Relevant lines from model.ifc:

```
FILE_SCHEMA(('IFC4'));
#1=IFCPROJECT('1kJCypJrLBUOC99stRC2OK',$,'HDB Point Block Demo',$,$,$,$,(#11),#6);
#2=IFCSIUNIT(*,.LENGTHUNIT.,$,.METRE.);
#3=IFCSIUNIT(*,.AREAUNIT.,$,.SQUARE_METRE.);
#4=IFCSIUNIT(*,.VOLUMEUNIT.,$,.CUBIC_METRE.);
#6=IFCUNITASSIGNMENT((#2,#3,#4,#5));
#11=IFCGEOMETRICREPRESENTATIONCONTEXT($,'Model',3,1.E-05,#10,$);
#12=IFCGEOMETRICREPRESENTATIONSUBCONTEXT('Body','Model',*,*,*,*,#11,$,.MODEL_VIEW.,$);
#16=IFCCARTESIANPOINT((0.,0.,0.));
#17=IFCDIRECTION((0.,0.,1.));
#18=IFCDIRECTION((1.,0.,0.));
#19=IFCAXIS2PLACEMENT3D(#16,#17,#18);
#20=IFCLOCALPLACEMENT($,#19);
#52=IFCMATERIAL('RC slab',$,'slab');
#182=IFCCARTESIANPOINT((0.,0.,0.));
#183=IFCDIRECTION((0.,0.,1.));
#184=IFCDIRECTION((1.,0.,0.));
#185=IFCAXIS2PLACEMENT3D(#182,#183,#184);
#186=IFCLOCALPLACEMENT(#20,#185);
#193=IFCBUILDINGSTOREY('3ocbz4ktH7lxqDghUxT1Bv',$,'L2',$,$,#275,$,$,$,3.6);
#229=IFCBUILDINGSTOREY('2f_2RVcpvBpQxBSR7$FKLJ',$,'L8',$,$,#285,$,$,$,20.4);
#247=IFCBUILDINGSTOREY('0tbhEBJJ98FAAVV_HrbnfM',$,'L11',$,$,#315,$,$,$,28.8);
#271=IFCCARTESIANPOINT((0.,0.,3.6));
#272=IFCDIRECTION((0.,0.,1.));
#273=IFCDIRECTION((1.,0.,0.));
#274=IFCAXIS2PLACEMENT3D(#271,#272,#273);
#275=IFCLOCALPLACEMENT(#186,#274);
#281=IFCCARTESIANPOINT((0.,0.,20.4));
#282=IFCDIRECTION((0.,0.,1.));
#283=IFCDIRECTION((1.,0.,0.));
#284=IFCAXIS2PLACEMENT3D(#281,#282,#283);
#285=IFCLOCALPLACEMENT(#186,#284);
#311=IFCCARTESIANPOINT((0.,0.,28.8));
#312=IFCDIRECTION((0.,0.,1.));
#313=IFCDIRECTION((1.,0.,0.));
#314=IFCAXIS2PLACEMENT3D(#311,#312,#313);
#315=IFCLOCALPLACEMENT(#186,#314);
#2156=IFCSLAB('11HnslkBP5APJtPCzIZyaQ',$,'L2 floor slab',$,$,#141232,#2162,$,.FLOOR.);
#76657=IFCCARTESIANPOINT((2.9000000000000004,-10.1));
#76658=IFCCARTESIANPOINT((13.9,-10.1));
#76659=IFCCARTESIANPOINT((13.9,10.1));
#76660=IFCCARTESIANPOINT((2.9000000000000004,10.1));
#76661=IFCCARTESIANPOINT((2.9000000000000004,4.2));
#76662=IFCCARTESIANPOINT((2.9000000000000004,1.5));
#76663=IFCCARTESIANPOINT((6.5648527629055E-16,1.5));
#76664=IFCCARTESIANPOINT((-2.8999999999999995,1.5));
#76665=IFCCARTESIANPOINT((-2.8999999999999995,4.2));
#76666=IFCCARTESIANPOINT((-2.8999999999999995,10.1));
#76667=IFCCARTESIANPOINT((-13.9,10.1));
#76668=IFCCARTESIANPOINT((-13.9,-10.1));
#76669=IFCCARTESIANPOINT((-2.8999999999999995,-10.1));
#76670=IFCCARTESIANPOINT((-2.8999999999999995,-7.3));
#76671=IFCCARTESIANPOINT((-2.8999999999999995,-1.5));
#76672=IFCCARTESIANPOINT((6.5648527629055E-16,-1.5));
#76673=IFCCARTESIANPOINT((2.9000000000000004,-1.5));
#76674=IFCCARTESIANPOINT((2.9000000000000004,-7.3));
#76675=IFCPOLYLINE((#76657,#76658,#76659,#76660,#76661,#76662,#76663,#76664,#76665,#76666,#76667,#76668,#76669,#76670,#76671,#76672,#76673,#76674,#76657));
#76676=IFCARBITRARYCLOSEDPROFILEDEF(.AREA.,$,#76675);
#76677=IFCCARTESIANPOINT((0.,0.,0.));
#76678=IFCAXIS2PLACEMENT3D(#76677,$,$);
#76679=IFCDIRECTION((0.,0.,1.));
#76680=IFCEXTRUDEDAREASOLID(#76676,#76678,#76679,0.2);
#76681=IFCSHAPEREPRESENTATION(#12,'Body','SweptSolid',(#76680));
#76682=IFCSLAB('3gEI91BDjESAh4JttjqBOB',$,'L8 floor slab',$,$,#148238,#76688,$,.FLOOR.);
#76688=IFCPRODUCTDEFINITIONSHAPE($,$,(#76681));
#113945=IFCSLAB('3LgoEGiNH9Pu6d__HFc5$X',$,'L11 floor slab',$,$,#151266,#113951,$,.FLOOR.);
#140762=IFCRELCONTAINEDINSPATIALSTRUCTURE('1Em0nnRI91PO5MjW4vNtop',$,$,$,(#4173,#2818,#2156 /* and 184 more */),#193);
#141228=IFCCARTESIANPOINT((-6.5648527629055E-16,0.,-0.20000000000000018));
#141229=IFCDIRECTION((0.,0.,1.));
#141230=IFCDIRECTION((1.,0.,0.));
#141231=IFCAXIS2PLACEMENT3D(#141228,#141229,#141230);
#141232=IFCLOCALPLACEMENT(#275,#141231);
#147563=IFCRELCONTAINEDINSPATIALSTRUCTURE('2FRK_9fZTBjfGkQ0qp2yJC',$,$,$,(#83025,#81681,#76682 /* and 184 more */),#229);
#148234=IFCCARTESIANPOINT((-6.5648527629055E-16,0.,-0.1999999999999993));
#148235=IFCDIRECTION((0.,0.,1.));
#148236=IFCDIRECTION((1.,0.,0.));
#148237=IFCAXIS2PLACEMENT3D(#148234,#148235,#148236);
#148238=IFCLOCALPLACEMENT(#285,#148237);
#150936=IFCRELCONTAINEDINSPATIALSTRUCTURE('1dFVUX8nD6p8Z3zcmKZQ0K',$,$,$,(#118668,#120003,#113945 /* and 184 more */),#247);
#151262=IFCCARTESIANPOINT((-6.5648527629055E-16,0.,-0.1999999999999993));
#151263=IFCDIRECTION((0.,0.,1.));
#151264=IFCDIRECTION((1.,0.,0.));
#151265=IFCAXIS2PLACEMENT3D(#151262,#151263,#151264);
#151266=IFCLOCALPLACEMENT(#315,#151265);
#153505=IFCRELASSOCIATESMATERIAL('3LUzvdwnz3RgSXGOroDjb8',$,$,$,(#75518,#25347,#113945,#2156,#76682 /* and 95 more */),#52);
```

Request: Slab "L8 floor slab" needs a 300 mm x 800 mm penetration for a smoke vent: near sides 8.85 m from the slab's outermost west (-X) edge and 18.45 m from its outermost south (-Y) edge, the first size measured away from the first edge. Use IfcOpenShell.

```python
import numpy as np
import ifcopenshell
import ifcopenshell.api.feature
import ifcopenshell.api.geometry
import ifcopenshell.api.root
import ifcopenshell.geom
import ifcopenshell.util.placement
import ifcopenshell.util.representation
import ifcopenshell.util.shape
import ifcopenshell.util.unit

model = ifcopenshell.open("model.ifc")
unit_scale = ifcopenshell.util.unit.calculate_unit_scale(model)
settings = ifcopenshell.geom.settings()


def volume(element):
    """Net volume in cubic metres, openings subtracted."""
    shape = ifcopenshell.geom.create_shape(settings, element)
    return ifcopenshell.util.shape.get_volume(shape.geometry)


slab = model.by_id(76682)
before = volume(slab)

# Extent in the slab's own axes, in metres. The edges named are its -X and -Y sides.
slab_shape = ifcopenshell.geom.create_shape(settings, slab)
vertices = ifcopenshell.util.shape.get_vertices(slab_shape.geometry)
x_min, y_min, bottom = vertices.min(axis=0)
top = vertices[:, 2].max()

opening = ifcopenshell.api.root.create_entity(model, ifc_class="IfcOpeningElement", name="Smoke vent opening", predefined_type="OPENING")
context = ifcopenshell.util.representation.get_context(model, "Model", "Body", "MODEL_VIEW")
width, depth = 0.3, 0.8
outline = [(0.0, 0.0), (width, 0.0), (width, depth), (0.0, depth), (0.0, 0.0)]
# Overshoot both faces by 50 mm so the cut is clean.
shape = ifcopenshell.api.geometry.add_slab_representation(
    model, context=context, depth=top - bottom + 0.1, polyline=outline
)
ifcopenshell.api.geometry.assign_representation(model, product=opening, representation=shape)

matrix = ifcopenshell.util.placement.get_local_placement(slab.ObjectPlacement)
matrix[:, 3] = matrix @ np.append(np.array([x_min + 8.85, y_min + 18.45, bottom - 0.05]) / unit_scale, 1.0)
ifcopenshell.api.geometry.edit_object_placement(model, product=opening, matrix=matrix, is_si=False)
ifcopenshell.api.feature.add_feature(model, feature=opening, element=slab)

after = volume(slab)

print(f"slab volume {before:.3f} -> {after:.3f} m3")

model.write("model_rev.ifc")
```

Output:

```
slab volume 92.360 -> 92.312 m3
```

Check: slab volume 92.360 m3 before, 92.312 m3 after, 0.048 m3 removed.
